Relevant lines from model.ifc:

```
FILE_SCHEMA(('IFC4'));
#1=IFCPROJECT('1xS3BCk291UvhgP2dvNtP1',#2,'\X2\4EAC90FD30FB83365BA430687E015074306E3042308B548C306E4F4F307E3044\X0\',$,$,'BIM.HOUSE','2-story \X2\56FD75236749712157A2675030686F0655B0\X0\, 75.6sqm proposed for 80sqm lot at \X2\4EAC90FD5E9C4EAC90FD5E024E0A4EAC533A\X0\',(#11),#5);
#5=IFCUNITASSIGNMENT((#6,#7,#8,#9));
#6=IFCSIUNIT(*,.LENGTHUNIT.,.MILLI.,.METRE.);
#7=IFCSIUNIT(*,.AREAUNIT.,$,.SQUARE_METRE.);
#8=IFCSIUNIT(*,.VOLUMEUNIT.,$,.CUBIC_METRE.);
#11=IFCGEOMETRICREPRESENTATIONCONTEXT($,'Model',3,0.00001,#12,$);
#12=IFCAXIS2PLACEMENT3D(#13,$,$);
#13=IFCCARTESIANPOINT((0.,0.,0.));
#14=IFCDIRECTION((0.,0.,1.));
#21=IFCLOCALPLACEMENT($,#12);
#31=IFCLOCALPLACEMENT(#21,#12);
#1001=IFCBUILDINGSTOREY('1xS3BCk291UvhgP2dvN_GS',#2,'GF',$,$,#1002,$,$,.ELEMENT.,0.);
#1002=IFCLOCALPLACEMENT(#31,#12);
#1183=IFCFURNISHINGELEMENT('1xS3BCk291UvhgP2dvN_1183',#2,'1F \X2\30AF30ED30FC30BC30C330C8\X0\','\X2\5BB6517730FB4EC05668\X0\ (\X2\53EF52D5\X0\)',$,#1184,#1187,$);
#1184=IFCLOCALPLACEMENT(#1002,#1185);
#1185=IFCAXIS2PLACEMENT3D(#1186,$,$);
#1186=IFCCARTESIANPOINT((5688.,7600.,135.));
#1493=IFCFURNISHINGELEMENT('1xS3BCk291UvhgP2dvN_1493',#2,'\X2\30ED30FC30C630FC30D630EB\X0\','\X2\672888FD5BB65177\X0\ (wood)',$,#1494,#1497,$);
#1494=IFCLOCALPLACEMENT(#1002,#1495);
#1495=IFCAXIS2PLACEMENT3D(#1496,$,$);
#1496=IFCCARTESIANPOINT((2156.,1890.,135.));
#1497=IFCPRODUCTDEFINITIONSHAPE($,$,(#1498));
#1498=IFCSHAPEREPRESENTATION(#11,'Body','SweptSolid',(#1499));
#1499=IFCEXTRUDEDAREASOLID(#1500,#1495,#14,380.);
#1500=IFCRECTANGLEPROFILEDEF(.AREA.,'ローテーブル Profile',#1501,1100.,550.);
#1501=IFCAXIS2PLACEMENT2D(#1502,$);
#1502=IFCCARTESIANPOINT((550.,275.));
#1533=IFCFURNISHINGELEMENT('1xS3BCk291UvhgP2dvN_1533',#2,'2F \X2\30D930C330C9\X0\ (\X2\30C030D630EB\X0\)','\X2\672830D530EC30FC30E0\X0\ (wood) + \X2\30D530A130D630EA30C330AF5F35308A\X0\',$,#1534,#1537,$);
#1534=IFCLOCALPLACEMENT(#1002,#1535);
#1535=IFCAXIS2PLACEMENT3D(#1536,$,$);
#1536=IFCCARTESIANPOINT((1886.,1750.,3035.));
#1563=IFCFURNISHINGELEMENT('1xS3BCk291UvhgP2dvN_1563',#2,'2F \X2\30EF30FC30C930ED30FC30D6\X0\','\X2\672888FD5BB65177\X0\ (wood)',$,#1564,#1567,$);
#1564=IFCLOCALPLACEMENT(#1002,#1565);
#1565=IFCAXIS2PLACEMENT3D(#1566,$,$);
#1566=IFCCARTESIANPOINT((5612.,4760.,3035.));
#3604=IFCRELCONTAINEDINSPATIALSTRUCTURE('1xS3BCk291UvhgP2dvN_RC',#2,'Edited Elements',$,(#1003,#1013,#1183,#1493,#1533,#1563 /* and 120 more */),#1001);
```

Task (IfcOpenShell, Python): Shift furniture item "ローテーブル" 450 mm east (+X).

```python
import ifcopenshell
import ifcopenshell.api.geometry
import ifcopenshell.util.placement
import ifcopenshell.util.unit

model = ifcopenshell.open("model.ifc")
unit_scale = ifcopenshell.util.unit.calculate_unit_scale(model)

item = model.by_guid("1xS3BCk291UvhgP2dvN_1493")
matrix = ifcopenshell.util.placement.get_local_placement(item.ObjectPlacement)
matrix[0, 3] += 0.45 / unit_scale
ifcopenshell.api.geometry.edit_object_placement(model, product=item, matrix=matrix, is_si=False)

print(ifcopenshell.util.placement.get_local_placement(item.ObjectPlacement).round(3) + 0.0)

model.write("model_edited.ifc")
```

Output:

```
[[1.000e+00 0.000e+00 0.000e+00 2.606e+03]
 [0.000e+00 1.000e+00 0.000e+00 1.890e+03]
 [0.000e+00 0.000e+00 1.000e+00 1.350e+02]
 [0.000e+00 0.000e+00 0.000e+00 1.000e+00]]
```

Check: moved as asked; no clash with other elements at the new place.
